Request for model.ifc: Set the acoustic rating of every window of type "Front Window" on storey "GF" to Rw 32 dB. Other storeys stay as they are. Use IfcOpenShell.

First a look at what the model holds.

```python
import ifcopenshell
import ifcopenshell.util.element

model = ifcopenshell.open("model.ifc")
print(model.schema)
storey = next(s for s in model.by_type("IfcBuildingStorey") if s.Name == "GF")
windows = [e for e in ifcopenshell.util.element.get_decomposition(storey) if e.is_a("IfcWindow")]
seen = {}
for e in windows:
    element_type = ifcopenshell.util.element.get_type(e)
    key = (element_type.Name if element_type != e and element_type else None, ifcopenshell.util.element.get_pset(e, "Pset_WindowCommon", "AcousticRating"))
    seen[key] = seen.get(key, 0) + 1
for (name, value), count in sorted(seen.items(), key=str):
    print(count, "x", name, "|", value)
```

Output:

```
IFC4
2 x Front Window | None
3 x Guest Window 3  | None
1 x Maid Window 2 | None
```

```python
import ifcopenshell
import ifcopenshell.api.pset
import ifcopenshell.util.element

model = ifcopenshell.open("model.ifc")

storey = next(s for s in model.by_type("IfcBuildingStorey") if s.Name == "GF")
windows = [e for e in ifcopenshell.util.element.get_decomposition(storey) if e.is_a("IfcWindow")]

count = 0
for e in windows:
    element_type = ifcopenshell.util.element.get_type(e)
    if element_type in (None, e) or element_type.Name != "Front Window":
        continue
    # add_pset returns the element's existing set when there is one.
    pset = ifcopenshell.api.pset.add_pset(model, product=e, name="Pset_WindowCommon")
    ifcopenshell.api.pset.edit_pset(model, pset=pset, properties={"AcousticRating": "Rw 32 dB"})
    count += 1

print(count, "windows updated")

model.write("model_updated.ifc")
```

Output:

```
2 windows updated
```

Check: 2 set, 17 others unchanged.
